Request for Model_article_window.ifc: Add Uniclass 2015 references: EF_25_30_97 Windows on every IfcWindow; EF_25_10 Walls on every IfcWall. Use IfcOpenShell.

First a look at what the model holds.

```python
import ifcopenshell

model = ifcopenshell.open("Model_article_window.ifc")
print(model.schema)
print("classifications:", [c.Name for c in model.by_type("IfcClassification")])
for ifc_class in ("IfcDoor", "IfcRoof", "IfcStair", "IfcWall", "IfcWindow"):
    print(ifc_class, len(model.by_type(ifc_class)))
```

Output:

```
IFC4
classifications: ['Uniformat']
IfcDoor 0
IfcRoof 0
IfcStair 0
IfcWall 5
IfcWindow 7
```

```python
import ifcopenshell
import ifcopenshell.api.classification

model = ifcopenshell.open("Model_article_window.ifc")

system = ifcopenshell.api.classification.add_classification(model, classification="Uniclass 2015")

codes = {
    "IfcWindow": ("EF_25_30_97", "Windows"),
    "IfcWall": ("EF_25_10", "Walls"),
}
for ifc_class, (code, name) in codes.items():
    products = model.by_type(ifc_class)
    ifcopenshell.api.classification.add_reference(
        model, products=products, classification=system, identification=code, name=name
    )
    print(code, len(products))

model.write("Model_article_window_rev.ifc")
```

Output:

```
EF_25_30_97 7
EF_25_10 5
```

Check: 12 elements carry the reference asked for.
